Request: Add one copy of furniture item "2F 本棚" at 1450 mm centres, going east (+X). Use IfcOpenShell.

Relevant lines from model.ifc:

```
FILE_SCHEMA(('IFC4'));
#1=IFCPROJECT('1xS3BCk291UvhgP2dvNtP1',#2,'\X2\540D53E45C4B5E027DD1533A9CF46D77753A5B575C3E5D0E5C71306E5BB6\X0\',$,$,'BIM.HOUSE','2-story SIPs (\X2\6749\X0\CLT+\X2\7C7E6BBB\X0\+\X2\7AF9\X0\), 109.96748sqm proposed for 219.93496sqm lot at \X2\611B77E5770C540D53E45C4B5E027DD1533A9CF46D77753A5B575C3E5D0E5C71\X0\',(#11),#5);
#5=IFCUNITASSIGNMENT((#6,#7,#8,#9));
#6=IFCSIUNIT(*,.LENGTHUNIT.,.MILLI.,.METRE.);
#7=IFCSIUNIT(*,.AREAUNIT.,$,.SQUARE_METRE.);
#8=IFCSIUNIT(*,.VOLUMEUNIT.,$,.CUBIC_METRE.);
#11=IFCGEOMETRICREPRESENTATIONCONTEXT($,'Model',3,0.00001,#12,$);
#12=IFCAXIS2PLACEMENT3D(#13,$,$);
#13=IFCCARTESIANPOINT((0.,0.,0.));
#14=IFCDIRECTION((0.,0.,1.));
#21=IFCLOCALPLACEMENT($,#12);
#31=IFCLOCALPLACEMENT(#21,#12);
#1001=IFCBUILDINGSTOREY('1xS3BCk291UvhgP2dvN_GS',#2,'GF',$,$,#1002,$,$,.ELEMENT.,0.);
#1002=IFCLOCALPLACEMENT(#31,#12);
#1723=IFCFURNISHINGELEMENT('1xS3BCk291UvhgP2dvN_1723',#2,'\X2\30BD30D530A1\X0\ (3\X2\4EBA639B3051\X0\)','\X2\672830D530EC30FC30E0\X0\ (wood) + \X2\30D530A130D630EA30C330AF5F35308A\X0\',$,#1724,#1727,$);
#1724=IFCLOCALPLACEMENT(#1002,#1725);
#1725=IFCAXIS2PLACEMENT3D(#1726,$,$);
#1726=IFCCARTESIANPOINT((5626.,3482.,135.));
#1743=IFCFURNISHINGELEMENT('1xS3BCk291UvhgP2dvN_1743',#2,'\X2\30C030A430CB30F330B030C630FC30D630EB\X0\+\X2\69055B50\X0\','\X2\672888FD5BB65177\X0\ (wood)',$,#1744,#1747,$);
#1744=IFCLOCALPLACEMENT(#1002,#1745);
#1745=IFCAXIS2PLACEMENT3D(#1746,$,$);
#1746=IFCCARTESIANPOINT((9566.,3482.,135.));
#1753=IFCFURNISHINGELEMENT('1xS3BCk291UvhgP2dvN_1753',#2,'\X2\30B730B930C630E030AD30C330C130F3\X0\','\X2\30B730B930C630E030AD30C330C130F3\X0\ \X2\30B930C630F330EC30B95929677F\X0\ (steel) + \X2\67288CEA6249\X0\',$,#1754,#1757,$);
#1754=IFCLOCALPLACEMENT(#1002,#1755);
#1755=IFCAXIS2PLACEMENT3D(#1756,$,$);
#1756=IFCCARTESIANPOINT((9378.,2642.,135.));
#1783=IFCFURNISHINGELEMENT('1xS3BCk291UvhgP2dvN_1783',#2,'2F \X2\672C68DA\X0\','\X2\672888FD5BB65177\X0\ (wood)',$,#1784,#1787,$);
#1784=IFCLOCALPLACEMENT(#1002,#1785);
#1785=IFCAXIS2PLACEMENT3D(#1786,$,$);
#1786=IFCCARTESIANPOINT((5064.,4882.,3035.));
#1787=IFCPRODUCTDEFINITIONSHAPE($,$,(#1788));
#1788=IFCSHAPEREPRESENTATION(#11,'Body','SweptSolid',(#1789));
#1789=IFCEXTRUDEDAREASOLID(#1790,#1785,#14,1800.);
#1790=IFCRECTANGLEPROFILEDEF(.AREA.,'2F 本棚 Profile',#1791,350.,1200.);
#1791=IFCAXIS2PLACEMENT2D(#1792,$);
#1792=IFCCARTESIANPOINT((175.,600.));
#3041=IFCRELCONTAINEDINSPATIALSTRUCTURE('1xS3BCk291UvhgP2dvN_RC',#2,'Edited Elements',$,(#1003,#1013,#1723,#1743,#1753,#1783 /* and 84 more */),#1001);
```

```python
import numpy as np
import ifcopenshell
import ifcopenshell.api.geometry
import ifcopenshell.api.root
import ifcopenshell.util.element
import ifcopenshell.util.placement

model = ifcopenshell.open("model.ifc")


def reuse_history(source, copy):
    """copy_class also copies each property set's owner history, people and application; keep the originals."""
    for rel in copy.IsDefinedBy:
        if rel.is_a("IfcRelDefinesByProperties") and (history := rel.RelatingPropertyDefinition.OwnerHistory):
            rel.RelatingPropertyDefinition.OwnerHistory = source.OwnerHistory
            ifcopenshell.util.element.remove_deep2(model, history)


source = model.by_id(1783)
base = ifcopenshell.util.placement.get_local_placement(source.ObjectPlacement)
step = np.array([1.0, 0.0, 0.0]) * 1450.0

for i in range(1, 2):
    copy = ifcopenshell.api.root.copy_class(model, product=source)
    copy.Representation = ifcopenshell.util.element.copy_deep(
        model, source.Representation, exclude=["IfcGeometricRepresentationContext", "IfcRepresentationMap"]
    )
    reuse_history(source, copy)
    matrix = base.copy()
    matrix[:3, 3] += i * step
    print("added at", matrix[:3, 3].round(3) + 0.0)
    ifcopenshell.api.geometry.edit_object_placement(model, product=copy, matrix=matrix, is_si=False)

model.write("model-out.ifc")
```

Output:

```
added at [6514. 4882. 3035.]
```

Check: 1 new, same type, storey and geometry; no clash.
